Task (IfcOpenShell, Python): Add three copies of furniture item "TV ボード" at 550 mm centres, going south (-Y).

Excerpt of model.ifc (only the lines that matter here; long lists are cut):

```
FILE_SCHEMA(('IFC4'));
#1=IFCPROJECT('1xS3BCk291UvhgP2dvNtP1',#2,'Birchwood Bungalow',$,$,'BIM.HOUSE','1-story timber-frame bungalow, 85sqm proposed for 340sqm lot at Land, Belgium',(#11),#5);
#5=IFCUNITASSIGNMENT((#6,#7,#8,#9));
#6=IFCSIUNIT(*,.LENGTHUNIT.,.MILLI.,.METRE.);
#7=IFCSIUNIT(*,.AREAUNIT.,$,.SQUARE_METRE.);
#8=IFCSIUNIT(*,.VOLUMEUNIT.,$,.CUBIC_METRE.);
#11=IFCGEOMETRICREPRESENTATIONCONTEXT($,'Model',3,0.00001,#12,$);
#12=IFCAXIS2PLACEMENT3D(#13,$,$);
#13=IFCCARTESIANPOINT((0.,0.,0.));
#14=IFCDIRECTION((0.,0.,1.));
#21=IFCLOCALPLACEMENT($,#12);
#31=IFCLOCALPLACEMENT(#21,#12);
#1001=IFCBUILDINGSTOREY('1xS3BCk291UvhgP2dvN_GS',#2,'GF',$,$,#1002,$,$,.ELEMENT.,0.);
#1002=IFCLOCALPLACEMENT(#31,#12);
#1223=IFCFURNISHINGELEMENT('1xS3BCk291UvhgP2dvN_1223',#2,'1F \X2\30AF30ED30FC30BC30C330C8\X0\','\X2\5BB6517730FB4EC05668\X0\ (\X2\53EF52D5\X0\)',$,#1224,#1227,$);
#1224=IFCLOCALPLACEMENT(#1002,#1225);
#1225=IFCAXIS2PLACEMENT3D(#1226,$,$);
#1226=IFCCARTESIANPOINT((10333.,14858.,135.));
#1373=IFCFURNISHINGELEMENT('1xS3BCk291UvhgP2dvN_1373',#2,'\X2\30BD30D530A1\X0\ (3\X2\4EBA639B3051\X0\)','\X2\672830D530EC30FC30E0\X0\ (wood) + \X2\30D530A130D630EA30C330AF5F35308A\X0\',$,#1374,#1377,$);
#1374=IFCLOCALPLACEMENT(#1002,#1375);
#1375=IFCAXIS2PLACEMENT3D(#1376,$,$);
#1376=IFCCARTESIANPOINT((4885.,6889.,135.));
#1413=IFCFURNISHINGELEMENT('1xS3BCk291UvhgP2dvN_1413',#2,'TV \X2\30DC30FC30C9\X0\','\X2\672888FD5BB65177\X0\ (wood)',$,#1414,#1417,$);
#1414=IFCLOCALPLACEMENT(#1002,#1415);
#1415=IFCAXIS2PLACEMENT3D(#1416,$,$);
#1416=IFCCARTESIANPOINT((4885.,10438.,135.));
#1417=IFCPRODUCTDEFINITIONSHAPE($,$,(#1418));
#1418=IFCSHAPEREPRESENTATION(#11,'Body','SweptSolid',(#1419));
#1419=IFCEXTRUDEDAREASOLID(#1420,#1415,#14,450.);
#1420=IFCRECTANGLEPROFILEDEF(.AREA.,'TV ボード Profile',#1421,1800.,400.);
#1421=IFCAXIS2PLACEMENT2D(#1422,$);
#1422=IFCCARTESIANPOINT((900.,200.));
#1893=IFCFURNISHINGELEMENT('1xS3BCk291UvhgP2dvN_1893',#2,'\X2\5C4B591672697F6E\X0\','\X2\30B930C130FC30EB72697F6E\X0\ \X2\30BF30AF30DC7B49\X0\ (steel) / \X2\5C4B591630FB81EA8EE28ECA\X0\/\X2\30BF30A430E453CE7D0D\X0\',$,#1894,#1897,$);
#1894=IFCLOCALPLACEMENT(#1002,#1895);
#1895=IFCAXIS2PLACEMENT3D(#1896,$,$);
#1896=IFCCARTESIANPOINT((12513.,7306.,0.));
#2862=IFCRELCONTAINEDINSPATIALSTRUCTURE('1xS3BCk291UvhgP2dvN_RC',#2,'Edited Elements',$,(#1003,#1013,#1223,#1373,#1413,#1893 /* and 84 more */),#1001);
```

```python
import numpy as np
import ifcopenshell
import ifcopenshell.api.geometry
import ifcopenshell.api.root
import ifcopenshell.util.element
import ifcopenshell.util.placement

model = ifcopenshell.open("model.ifc")


def reuse_history(source, copy):
    """copy_class also copies each property set's owner history, people and application; keep the originals."""
    for rel in copy.IsDefinedBy:
        if rel.is_a("IfcRelDefinesByProperties") and (history := rel.RelatingPropertyDefinition.OwnerHistory):
            rel.RelatingPropertyDefinition.OwnerHistory = source.OwnerHistory
            ifcopenshell.util.element.remove_deep2(model, history)


source = model.by_id(1413)
base = ifcopenshell.util.placement.get_local_placement(source.ObjectPlacement)
step = np.array([0.0, -1.0, 0.0]) * 550.0

for i in range(1, 4):
    copy = ifcopenshell.api.root.copy_class(model, product=source)
    copy.Representation = ifcopenshell.util.element.copy_deep(
        model, source.Representation, exclude=["IfcGeometricRepresentationContext", "IfcRepresentationMap"]
    )
    reuse_history(source, copy)
    matrix = base.copy()
    matrix[:3, 3] += i * step
    print("added at", matrix[:3, 3].round(3) + 0.0)
    ifcopenshell.api.geometry.edit_object_placement(model, product=copy, matrix=matrix, is_si=False)

model.write("model_edited.ifc")
```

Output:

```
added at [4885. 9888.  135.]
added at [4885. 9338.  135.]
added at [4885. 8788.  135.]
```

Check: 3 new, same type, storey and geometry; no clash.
